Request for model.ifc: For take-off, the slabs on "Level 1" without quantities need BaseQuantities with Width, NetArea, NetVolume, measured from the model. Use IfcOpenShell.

First a look at what the model holds.

```python
import ifcopenshell
import ifcopenshell.util.element
import ifcopenshell.util.unit

model = ifcopenshell.open("model.ifc")
print(model.schema)
for unit_type in ("LENGTHUNIT", "AREAUNIT", "VOLUMEUNIT"):
    print(unit_type, ifcopenshell.util.unit.calculate_unit_scale(model, unit_type))
storey = next(s for s in model.by_type("IfcBuildingStorey") if s.Name == "Level 1")
slabs = [e for e in ifcopenshell.util.element.get_decomposition(storey) if e.is_a("IfcSlab")]
for e in sorted(slabs, key=lambda e: e.id()):
    print(e.id(), e.is_a(), e.Name, list(ifcopenshell.util.element.get_psets(e, qtos_only=True)), sep=" | ")
```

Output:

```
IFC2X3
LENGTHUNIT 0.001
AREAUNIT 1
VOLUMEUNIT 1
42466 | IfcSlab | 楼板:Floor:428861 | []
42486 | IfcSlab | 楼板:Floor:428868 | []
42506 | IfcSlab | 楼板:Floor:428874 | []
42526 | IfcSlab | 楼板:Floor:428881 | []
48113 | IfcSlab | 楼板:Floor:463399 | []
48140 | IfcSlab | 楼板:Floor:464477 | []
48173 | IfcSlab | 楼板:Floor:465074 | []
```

```python
import ifcopenshell
import ifcopenshell.api.pset
import ifcopenshell.geom
import ifcopenshell.util.element
import ifcopenshell.util.shape
import ifcopenshell.util.unit

model = ifcopenshell.open("model.ifc")
unit_scale = ifcopenshell.util.unit.calculate_unit_scale(model)
area_scale = ifcopenshell.util.unit.calculate_unit_scale(model, "AREAUNIT")
volume_scale = ifcopenshell.util.unit.calculate_unit_scale(model, "VOLUMEUNIT")
settings = ifcopenshell.geom.settings()

storey = next(s for s in model.by_type("IfcBuildingStorey") if s.Name == "Level 1")
slabs = [e for e in ifcopenshell.util.element.get_decomposition(storey) if e.is_a("IfcSlab")]

for e in sorted(slabs, key=lambda e: e.id()):
    if ifcopenshell.util.element.get_psets(e, qtos_only=True, should_inherit=False):
        continue
    # Geometry comes back in metres, in the element's own axes.
    shape = ifcopenshell.geom.create_shape(settings, e)
    values = {
        "Width": ifcopenshell.util.shape.get_z(shape.geometry) / unit_scale,
        "NetArea": ifcopenshell.util.shape.get_footprint_area(shape.geometry) / area_scale,
        "NetVolume": ifcopenshell.util.shape.get_volume(shape.geometry) / volume_scale,
    }
    qto = ifcopenshell.api.pset.add_qto(model, product=e, name="BaseQuantities")
    ifcopenshell.api.pset.edit_qto(model, qto=qto, properties=values)
    print(e.id(), {k: round(v, 3) for k, v in values.items()})

model.write("model_updated.ifc")
```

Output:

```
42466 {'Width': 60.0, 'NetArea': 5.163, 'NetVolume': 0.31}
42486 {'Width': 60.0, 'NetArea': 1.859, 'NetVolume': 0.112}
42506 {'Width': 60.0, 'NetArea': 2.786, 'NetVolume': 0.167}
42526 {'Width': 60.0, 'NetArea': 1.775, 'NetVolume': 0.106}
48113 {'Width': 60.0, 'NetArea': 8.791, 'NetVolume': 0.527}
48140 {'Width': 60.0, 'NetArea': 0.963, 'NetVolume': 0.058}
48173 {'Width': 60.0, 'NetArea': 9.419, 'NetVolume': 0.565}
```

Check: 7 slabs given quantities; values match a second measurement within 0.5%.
